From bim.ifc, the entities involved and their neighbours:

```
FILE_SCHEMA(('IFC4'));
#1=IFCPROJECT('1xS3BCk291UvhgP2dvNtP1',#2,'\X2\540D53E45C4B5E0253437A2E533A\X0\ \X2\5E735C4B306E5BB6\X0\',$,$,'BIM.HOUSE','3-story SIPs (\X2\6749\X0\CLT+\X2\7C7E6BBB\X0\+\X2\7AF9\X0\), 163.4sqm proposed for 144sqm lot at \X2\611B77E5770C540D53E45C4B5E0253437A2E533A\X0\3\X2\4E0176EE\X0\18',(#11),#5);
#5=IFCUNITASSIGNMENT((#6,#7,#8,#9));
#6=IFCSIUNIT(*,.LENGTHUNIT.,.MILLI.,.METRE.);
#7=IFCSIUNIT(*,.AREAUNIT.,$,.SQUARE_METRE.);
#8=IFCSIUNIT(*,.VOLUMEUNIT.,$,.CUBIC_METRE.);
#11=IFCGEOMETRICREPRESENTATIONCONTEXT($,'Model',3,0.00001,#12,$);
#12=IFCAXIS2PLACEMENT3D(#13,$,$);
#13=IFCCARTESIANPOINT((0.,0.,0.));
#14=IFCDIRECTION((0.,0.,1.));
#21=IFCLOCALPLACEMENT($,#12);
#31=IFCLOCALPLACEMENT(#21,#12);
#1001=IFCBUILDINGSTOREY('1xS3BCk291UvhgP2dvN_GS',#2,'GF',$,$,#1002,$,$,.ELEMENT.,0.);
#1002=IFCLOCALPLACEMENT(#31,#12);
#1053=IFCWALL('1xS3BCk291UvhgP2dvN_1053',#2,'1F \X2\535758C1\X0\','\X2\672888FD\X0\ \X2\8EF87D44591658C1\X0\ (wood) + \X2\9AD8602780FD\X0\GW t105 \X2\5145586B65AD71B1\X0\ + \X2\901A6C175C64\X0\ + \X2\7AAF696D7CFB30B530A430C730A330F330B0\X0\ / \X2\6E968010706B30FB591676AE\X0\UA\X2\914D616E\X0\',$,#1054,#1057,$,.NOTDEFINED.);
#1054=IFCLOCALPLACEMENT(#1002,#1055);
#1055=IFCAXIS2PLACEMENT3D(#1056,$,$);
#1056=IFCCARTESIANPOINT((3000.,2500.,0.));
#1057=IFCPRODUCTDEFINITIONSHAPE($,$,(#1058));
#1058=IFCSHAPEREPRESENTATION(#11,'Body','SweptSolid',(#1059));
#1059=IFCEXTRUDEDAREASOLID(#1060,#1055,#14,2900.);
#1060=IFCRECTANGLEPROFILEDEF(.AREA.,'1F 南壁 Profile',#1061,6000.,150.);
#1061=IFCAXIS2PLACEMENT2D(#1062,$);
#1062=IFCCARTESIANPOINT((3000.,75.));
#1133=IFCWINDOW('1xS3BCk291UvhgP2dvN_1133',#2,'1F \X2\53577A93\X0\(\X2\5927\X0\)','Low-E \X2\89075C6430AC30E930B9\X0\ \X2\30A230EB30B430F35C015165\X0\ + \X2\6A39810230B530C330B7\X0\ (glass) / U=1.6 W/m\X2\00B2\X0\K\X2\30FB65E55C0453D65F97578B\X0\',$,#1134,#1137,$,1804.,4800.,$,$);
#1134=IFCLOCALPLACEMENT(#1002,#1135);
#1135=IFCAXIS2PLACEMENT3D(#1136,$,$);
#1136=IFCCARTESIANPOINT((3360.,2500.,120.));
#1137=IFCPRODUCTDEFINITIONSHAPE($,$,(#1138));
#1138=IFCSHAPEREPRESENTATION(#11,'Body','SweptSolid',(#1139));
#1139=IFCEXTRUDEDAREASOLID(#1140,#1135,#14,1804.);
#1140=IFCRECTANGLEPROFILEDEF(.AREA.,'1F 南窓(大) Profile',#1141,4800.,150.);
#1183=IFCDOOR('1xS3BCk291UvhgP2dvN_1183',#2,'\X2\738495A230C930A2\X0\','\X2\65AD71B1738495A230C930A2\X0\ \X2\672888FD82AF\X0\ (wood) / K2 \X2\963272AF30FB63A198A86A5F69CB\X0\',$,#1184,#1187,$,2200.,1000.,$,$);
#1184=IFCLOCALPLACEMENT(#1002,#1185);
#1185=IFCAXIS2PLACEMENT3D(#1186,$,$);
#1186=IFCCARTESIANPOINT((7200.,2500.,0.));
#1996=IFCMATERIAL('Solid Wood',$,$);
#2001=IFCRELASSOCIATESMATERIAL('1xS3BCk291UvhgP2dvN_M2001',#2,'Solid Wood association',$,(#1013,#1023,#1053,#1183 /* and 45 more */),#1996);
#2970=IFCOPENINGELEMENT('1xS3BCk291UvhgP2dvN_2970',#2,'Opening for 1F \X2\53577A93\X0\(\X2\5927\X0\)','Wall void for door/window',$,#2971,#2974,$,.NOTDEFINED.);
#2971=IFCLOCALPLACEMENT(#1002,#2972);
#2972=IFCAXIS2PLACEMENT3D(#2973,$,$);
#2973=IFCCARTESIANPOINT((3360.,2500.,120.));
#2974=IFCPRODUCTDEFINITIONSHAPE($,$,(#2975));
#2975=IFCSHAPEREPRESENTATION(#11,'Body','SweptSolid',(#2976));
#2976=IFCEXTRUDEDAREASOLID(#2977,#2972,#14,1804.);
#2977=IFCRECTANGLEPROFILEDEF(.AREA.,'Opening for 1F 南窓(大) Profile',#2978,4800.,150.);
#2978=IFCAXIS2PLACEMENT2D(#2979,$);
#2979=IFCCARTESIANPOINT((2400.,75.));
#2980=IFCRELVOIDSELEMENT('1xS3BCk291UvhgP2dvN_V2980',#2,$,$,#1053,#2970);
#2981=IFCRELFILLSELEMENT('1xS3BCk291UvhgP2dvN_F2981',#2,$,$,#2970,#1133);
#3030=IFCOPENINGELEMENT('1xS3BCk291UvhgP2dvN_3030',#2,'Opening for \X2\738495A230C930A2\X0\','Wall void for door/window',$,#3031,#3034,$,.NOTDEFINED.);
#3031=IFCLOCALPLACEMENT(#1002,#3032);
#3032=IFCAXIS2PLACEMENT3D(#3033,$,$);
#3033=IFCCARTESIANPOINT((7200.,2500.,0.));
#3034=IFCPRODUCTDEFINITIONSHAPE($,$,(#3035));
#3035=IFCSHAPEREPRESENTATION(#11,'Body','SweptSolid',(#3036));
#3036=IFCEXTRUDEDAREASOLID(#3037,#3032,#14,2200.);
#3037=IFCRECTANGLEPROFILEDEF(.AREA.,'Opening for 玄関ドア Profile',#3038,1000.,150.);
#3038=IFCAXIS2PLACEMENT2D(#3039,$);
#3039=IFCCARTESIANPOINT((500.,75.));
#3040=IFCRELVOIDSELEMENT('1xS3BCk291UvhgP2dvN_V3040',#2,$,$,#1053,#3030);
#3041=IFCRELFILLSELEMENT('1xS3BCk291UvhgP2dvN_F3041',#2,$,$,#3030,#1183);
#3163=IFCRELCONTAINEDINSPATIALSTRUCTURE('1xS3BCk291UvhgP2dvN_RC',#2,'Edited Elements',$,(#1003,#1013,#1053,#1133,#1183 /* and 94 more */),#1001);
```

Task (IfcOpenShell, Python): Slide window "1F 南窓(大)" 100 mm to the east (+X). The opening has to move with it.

```python
import ifcopenshell
import ifcopenshell.api.geometry
import ifcopenshell.util.placement
import ifcopenshell.util.unit

model = ifcopenshell.open("bim.ifc")
unit_scale = ifcopenshell.util.unit.calculate_unit_scale(model)

window = model.by_id(1133)
opening = window.FillsVoids[0].RelatingOpeningElement
wall = opening.VoidsElements[0].RelatingBuildingElement

wall_matrix = ifcopenshell.util.placement.get_local_placement(wall.ObjectPlacement)
shift = wall_matrix[:3, 0] * 0.1 / unit_scale
before = ifcopenshell.util.placement.get_local_placement(window.ObjectPlacement)[:3, 3].copy()

# The window is not placed relative to its opening, so move both.
for product in (opening, window):
    matrix = ifcopenshell.util.placement.get_local_placement(product.ObjectPlacement)
    matrix[:3, 3] += shift
    ifcopenshell.api.geometry.edit_object_placement(model, product=product, matrix=matrix, is_si=False)

after = ifcopenshell.util.placement.get_local_placement(window.ObjectPlacement)[:3, 3]
print("window moved by", (after - before).round(3) + 0.0)

model.write("bim_rev.ifc")
```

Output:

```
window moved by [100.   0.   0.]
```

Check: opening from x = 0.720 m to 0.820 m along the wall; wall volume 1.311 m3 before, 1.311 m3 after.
